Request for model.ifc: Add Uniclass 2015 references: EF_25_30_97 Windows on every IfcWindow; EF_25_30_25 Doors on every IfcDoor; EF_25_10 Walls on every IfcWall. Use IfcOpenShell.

First a look at what the model holds.

```python
import ifcopenshell

model = ifcopenshell.open("model.ifc")
print(model.schema)
print("classifications:", [c.Name for c in model.by_type("IfcClassification")])
for ifc_class in ("IfcDoor", "IfcRoof", "IfcStair", "IfcWall", "IfcWindow"):
    print(ifc_class, len(model.by_type(ifc_class)))
```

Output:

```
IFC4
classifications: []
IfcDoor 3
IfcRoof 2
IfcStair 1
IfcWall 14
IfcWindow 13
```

```python
import ifcopenshell
import ifcopenshell.api.classification

model = ifcopenshell.open("model.ifc")

system = ifcopenshell.api.classification.add_classification(model, classification="Uniclass 2015")

codes = {
    "IfcWindow": ("EF_25_30_97", "Windows"),
    "IfcDoor": ("EF_25_30_25", "Doors"),
    "IfcWall": ("EF_25_10", "Walls"),
}
for ifc_class, (code, name) in codes.items():
    products = model.by_type(ifc_class)
    ifcopenshell.api.classification.add_reference(
        model, products=products, classification=system, identification=code, name=name
    )
    print(code, len(products))

model.write("model_rev.ifc")
```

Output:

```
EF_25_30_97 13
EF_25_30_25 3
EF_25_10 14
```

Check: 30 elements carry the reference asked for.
